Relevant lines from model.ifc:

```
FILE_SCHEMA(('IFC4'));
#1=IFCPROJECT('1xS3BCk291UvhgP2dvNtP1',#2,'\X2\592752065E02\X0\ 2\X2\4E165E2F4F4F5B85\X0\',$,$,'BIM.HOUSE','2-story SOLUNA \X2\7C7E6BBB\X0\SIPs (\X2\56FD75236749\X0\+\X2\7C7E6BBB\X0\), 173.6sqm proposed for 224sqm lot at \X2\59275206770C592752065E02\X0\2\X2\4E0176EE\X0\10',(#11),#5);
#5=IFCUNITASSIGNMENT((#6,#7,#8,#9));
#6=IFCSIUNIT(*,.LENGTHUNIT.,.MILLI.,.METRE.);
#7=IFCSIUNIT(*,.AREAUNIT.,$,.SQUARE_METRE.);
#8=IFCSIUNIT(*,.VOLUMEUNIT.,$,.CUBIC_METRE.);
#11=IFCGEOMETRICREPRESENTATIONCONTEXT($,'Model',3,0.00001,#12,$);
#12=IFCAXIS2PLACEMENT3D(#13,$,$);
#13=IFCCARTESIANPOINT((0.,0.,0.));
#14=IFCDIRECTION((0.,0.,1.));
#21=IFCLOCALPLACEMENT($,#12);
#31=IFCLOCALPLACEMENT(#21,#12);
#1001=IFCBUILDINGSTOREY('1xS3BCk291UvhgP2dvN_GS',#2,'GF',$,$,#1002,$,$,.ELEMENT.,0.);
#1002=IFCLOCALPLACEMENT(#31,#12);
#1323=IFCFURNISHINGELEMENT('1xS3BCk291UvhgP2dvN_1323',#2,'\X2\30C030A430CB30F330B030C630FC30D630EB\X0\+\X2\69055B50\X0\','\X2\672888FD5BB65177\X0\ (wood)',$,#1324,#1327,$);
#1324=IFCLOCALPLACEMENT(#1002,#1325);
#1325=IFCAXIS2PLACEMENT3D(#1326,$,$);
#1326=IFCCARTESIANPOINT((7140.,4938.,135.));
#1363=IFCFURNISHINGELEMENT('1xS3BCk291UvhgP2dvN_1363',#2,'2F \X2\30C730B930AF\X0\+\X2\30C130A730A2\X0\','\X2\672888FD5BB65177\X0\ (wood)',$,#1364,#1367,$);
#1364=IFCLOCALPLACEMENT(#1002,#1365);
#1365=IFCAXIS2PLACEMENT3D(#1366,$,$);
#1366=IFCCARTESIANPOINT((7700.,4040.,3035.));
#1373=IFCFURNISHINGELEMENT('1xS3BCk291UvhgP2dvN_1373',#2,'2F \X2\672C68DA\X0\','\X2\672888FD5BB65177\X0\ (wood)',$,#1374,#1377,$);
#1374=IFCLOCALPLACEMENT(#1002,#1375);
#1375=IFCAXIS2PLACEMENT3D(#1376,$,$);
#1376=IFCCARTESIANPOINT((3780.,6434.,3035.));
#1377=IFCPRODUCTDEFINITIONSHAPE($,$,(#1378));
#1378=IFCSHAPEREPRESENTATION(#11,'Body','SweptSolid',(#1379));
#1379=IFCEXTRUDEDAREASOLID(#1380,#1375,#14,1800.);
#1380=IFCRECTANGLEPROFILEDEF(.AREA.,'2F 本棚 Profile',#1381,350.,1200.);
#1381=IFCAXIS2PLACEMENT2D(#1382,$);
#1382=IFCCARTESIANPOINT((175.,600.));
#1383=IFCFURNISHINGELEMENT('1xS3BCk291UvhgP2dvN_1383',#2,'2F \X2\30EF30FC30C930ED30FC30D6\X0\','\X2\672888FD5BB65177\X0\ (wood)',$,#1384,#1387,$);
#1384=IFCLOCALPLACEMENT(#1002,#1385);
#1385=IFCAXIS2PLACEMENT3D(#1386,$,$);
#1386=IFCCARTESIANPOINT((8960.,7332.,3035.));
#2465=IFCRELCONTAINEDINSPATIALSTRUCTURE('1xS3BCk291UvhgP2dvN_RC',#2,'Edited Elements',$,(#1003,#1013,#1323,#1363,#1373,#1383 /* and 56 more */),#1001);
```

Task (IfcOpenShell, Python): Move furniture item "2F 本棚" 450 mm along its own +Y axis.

```python
import ifcopenshell
import ifcopenshell.api.geometry
import ifcopenshell.util.placement

model = ifcopenshell.open("model.ifc")

item = model.by_guid("1xS3BCk291UvhgP2dvN_1373")
matrix = ifcopenshell.util.placement.get_local_placement(item.ObjectPlacement)
matrix[:3, 3] += matrix[:3, 1] * 450.0
ifcopenshell.api.geometry.edit_object_placement(model, product=item, matrix=matrix, is_si=False)

print(ifcopenshell.util.placement.get_local_placement(item.ObjectPlacement).round(3) + 0.0)

model.write("model_edited.ifc")
```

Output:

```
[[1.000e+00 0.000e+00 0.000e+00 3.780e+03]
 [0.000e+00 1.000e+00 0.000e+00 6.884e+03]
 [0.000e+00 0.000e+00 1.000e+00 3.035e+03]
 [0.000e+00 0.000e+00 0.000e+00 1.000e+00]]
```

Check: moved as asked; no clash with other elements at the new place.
